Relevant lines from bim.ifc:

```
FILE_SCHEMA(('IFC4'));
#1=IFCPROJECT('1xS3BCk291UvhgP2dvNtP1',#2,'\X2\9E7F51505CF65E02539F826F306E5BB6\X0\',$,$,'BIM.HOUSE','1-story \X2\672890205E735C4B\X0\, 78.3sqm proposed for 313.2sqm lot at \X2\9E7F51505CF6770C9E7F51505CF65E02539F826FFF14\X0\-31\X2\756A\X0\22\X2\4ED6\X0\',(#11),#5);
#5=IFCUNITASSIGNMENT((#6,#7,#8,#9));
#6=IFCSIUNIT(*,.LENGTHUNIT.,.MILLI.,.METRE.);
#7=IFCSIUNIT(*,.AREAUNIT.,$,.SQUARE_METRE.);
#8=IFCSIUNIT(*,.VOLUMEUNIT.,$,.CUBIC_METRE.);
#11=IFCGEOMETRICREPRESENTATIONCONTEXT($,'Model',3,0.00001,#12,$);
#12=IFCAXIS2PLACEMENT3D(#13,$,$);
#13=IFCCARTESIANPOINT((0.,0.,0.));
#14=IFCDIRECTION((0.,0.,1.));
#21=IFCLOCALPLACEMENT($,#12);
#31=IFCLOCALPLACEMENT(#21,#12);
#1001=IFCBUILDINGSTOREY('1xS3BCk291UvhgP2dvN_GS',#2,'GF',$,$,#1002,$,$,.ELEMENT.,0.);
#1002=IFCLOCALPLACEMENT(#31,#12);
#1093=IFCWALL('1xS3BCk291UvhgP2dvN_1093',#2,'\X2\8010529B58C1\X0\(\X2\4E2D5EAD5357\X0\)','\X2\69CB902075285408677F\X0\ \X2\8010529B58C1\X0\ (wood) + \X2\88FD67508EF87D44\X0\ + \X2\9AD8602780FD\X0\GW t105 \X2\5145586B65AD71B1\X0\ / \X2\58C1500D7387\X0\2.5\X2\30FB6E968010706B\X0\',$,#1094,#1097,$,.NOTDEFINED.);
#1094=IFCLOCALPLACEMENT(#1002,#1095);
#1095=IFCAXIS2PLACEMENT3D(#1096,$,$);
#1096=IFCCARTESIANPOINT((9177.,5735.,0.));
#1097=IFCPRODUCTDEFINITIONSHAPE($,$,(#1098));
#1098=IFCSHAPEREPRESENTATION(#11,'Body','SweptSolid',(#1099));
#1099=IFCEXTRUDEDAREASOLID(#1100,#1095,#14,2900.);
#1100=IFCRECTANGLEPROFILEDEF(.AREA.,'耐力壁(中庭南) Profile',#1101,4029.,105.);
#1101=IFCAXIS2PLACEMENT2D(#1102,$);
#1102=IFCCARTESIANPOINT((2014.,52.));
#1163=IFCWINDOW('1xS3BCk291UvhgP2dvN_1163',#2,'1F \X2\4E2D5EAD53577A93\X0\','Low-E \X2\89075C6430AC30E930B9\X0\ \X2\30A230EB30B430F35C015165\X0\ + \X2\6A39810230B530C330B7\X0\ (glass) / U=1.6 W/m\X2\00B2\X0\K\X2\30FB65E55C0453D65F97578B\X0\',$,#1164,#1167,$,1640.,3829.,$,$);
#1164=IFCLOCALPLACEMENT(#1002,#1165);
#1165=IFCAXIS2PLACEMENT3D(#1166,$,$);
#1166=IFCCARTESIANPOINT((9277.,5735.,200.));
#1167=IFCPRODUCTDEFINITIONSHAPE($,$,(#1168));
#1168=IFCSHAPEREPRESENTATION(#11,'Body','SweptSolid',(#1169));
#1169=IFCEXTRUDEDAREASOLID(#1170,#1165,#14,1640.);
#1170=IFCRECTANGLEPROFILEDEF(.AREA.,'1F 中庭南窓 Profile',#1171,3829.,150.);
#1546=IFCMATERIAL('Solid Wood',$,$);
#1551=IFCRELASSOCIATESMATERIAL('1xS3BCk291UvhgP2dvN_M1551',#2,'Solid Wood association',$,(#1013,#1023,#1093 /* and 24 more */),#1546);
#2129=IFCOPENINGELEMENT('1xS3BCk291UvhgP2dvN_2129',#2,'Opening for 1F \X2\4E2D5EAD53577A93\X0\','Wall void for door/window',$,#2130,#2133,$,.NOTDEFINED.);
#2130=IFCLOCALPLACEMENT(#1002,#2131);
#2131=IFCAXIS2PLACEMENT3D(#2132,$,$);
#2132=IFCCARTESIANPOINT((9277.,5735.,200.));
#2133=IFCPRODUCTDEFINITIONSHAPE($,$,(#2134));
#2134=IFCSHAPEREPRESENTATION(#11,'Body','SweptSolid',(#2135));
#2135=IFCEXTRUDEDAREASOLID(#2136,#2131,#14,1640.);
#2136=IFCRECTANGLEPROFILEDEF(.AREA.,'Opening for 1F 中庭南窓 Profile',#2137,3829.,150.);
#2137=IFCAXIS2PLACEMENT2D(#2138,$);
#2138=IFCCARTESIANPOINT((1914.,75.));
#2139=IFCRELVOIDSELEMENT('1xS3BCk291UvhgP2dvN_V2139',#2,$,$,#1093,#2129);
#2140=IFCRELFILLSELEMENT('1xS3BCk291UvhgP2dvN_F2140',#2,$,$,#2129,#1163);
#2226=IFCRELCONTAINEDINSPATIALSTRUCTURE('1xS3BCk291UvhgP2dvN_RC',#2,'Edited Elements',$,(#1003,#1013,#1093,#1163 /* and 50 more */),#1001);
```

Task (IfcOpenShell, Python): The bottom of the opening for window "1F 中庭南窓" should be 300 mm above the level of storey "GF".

```python
import numpy as np
import ifcopenshell
import ifcopenshell.api.geometry
import ifcopenshell.geom
import ifcopenshell.util.element
import ifcopenshell.util.placement
import ifcopenshell.util.shape
import ifcopenshell.util.unit

model = ifcopenshell.open("bim.ifc")
unit_scale = ifcopenshell.util.unit.calculate_unit_scale(model)

window = model.by_guid("1xS3BCk291UvhgP2dvN_1163")
opening = window.FillsVoids[0].RelatingOpeningElement
storey = ifcopenshell.util.element.get_container(window, ifc_class="IfcBuildingStorey")
level = ifcopenshell.util.placement.get_local_placement(storey.ObjectPlacement)[2, 3]

# The opening's origin need not be at the sill, so measure its lowest point.
shape = ifcopenshell.geom.create_shape(ifcopenshell.geom.settings(), opening)
bottom = ifcopenshell.util.shape.get_shape_bottom_elevation(shape, shape.geometry) / unit_scale
dz = level + 0.3 / unit_scale - bottom

shift = np.array([0.0, 0.0, dz])
# The window is not placed relative to its opening, so move both.
for product in (opening, window):
    matrix = ifcopenshell.util.placement.get_local_placement(product.ObjectPlacement)
    matrix[:3, 3] += shift
    ifcopenshell.api.geometry.edit_object_placement(model, product=product, matrix=matrix, is_si=False)

print(f"moved by {dz * unit_scale:+.3f} m")

model.write("bim_rev.ifc")
```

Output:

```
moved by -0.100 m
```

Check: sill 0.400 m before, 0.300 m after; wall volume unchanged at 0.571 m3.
